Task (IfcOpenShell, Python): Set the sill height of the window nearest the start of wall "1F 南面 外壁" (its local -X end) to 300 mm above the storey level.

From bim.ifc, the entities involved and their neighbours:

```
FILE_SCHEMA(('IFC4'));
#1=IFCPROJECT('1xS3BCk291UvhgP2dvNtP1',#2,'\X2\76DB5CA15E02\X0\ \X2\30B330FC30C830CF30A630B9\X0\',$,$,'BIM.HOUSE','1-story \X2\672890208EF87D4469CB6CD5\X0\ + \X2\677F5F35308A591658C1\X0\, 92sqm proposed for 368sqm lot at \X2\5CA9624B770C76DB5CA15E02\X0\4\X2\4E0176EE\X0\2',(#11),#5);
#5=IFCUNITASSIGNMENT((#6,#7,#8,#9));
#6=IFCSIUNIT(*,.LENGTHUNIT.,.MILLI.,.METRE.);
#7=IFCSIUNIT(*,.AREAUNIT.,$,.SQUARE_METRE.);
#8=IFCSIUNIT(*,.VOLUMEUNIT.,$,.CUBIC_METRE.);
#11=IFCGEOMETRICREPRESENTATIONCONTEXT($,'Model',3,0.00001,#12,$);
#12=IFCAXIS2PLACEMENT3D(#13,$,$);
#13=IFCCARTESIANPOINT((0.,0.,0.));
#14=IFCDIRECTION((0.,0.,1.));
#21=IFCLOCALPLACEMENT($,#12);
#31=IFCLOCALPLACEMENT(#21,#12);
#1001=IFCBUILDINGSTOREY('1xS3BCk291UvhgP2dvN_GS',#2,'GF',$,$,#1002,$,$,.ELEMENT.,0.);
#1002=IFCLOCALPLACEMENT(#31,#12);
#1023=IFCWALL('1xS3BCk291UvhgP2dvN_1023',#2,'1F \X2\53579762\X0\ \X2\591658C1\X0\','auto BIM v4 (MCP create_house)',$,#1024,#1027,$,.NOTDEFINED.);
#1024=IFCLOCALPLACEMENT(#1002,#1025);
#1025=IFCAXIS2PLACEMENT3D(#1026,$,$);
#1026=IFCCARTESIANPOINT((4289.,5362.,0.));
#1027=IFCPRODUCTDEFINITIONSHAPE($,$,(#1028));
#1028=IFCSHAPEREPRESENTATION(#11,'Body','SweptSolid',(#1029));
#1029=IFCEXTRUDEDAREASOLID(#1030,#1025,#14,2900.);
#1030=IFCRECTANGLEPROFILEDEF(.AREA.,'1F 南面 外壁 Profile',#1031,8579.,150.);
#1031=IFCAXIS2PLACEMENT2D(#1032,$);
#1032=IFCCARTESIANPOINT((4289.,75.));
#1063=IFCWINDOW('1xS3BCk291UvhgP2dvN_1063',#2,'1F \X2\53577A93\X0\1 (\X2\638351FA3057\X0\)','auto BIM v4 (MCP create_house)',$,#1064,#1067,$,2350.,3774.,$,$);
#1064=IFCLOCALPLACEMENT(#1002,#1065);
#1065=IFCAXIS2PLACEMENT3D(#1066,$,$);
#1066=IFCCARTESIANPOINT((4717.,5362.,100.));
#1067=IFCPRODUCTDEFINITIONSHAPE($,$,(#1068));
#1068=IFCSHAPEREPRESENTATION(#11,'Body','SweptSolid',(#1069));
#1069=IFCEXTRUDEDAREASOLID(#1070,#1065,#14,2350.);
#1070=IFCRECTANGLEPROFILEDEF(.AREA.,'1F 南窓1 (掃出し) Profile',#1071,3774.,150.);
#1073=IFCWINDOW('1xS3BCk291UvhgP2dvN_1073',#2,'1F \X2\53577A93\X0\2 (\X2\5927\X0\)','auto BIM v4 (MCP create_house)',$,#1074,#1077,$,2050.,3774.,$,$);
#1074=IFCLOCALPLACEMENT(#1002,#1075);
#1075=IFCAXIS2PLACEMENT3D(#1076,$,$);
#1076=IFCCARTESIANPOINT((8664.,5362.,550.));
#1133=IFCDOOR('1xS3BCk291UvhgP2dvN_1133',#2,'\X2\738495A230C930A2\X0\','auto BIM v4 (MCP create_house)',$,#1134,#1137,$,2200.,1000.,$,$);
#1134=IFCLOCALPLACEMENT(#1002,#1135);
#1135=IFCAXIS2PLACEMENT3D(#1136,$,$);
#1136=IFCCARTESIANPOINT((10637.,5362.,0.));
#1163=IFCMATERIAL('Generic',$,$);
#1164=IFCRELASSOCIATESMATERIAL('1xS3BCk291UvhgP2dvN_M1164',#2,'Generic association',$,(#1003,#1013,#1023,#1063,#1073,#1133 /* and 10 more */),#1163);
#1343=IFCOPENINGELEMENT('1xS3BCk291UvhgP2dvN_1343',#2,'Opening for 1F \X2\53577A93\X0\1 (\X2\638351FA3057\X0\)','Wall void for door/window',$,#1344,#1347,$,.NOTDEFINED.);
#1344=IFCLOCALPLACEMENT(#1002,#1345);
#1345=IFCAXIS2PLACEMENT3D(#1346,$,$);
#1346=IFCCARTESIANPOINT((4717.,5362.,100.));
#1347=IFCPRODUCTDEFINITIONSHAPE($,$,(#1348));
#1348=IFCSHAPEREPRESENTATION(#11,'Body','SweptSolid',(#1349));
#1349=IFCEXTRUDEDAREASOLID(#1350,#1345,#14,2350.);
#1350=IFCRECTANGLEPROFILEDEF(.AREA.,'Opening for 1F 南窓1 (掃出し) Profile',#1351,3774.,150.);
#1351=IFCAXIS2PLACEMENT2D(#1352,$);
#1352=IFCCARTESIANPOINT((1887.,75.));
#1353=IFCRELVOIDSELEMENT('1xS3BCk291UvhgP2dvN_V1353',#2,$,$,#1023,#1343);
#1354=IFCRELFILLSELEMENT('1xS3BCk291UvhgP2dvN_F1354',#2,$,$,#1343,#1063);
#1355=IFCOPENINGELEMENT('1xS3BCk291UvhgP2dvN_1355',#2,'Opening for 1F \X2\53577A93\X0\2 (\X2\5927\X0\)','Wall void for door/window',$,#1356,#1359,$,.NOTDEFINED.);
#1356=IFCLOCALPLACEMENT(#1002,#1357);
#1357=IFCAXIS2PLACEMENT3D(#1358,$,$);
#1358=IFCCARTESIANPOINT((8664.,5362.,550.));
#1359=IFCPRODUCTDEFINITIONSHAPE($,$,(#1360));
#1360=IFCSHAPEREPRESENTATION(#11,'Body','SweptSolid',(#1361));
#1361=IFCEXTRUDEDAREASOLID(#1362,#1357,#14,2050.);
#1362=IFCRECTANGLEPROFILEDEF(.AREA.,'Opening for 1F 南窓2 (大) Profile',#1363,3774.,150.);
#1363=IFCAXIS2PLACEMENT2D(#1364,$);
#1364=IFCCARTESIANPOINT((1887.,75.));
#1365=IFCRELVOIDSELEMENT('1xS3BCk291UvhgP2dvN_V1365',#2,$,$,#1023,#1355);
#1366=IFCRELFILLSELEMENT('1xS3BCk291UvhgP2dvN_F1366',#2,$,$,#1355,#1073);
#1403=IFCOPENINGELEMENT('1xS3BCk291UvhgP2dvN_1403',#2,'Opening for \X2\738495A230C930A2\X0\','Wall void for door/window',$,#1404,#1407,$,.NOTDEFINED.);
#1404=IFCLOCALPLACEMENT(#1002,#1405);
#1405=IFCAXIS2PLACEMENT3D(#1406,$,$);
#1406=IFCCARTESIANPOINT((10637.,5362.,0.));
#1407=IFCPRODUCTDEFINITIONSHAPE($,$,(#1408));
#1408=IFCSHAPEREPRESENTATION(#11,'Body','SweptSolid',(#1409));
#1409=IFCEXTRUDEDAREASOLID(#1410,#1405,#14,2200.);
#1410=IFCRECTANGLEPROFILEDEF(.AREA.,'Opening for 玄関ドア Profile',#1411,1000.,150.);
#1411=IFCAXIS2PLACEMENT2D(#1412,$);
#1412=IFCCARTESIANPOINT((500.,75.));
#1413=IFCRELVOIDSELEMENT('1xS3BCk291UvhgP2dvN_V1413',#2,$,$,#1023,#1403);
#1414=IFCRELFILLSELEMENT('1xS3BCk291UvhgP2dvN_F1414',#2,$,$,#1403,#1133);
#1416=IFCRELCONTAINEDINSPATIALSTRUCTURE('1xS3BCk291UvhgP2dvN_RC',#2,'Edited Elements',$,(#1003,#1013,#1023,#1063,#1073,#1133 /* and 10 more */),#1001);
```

```python
import numpy as np
import ifcopenshell
import ifcopenshell.api.geometry
import ifcopenshell.geom
import ifcopenshell.util.element
import ifcopenshell.util.placement
import ifcopenshell.util.shape
import ifcopenshell.util.unit

model = ifcopenshell.open("bim.ifc")
unit_scale = ifcopenshell.util.unit.calculate_unit_scale(model)

window = model.by_id(1063)
opening = window.FillsVoids[0].RelatingOpeningElement
storey = ifcopenshell.util.element.get_container(window, ifc_class="IfcBuildingStorey")
level = ifcopenshell.util.placement.get_local_placement(storey.ObjectPlacement)[2, 3]

# The opening's origin need not be at the sill, so measure its lowest point.
shape = ifcopenshell.geom.create_shape(ifcopenshell.geom.settings(), opening)
bottom = ifcopenshell.util.shape.get_shape_bottom_elevation(shape, shape.geometry) / unit_scale
dz = level + 300.0 - bottom

shift = np.array([0.0, 0.0, dz])
# The window is not placed relative to its opening, so move both.
for product in (opening, window):
    matrix = ifcopenshell.util.placement.get_local_placement(product.ObjectPlacement)
    matrix[:3, 3] += shift
    ifcopenshell.api.geometry.edit_object_placement(model, product=product, matrix=matrix, is_si=False)

print(f"moved by {dz * unit_scale:+.3f} m")

model.write("bim-out.ifc")
```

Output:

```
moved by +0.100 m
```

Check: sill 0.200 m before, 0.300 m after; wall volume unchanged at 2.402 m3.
